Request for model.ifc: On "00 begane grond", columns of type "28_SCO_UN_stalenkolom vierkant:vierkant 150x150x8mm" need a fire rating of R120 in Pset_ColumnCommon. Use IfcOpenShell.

First a look at what the model holds.

```python
import ifcopenshell
import ifcopenshell.util.element

model = ifcopenshell.open("model.ifc")
print(model.schema)
storey = next(s for s in model.by_type("IfcBuildingStorey") if s.Name == "00 begane grond")
columns = [e for e in ifcopenshell.util.element.get_decomposition(storey) if e.is_a("IfcColumn")]
seen = {}
for e in columns:
    element_type = ifcopenshell.util.element.get_type(e)
    key = (element_type.Name if element_type != e and element_type else None, ifcopenshell.util.element.get_pset(e, "Pset_ColumnCommon", "FireRating"))
    seen[key] = seen.get(key, 0) + 1
for (name, value), count in sorted(seen.items(), key=str):
    print(count, "x", name, "|", value)
```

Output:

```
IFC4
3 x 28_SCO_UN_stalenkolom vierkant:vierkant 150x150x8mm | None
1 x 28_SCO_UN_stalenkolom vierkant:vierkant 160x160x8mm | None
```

```python
import ifcopenshell
import ifcopenshell.api.pset
import ifcopenshell.util.element

model = ifcopenshell.open("model.ifc")

storey = next(s for s in model.by_type("IfcBuildingStorey") if s.Name == "00 begane grond")
columns = [e for e in ifcopenshell.util.element.get_decomposition(storey) if e.is_a("IfcColumn")]

count = 0
for e in columns:
    element_type = ifcopenshell.util.element.get_type(e)
    if element_type in (None, e) or element_type.Name != "28_SCO_UN_stalenkolom vierkant:vierkant 150x150x8mm":
        continue
    # add_pset returns the element's existing set when there is one.
    pset = ifcopenshell.api.pset.add_pset(model, product=e, name="Pset_ColumnCommon")
    ifcopenshell.api.pset.edit_pset(model, pset=pset, properties={"FireRating": "R120"})
    count += 1

print(count, "columns updated")

model.write("model-out.ifc")
```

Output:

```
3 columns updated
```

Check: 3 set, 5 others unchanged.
